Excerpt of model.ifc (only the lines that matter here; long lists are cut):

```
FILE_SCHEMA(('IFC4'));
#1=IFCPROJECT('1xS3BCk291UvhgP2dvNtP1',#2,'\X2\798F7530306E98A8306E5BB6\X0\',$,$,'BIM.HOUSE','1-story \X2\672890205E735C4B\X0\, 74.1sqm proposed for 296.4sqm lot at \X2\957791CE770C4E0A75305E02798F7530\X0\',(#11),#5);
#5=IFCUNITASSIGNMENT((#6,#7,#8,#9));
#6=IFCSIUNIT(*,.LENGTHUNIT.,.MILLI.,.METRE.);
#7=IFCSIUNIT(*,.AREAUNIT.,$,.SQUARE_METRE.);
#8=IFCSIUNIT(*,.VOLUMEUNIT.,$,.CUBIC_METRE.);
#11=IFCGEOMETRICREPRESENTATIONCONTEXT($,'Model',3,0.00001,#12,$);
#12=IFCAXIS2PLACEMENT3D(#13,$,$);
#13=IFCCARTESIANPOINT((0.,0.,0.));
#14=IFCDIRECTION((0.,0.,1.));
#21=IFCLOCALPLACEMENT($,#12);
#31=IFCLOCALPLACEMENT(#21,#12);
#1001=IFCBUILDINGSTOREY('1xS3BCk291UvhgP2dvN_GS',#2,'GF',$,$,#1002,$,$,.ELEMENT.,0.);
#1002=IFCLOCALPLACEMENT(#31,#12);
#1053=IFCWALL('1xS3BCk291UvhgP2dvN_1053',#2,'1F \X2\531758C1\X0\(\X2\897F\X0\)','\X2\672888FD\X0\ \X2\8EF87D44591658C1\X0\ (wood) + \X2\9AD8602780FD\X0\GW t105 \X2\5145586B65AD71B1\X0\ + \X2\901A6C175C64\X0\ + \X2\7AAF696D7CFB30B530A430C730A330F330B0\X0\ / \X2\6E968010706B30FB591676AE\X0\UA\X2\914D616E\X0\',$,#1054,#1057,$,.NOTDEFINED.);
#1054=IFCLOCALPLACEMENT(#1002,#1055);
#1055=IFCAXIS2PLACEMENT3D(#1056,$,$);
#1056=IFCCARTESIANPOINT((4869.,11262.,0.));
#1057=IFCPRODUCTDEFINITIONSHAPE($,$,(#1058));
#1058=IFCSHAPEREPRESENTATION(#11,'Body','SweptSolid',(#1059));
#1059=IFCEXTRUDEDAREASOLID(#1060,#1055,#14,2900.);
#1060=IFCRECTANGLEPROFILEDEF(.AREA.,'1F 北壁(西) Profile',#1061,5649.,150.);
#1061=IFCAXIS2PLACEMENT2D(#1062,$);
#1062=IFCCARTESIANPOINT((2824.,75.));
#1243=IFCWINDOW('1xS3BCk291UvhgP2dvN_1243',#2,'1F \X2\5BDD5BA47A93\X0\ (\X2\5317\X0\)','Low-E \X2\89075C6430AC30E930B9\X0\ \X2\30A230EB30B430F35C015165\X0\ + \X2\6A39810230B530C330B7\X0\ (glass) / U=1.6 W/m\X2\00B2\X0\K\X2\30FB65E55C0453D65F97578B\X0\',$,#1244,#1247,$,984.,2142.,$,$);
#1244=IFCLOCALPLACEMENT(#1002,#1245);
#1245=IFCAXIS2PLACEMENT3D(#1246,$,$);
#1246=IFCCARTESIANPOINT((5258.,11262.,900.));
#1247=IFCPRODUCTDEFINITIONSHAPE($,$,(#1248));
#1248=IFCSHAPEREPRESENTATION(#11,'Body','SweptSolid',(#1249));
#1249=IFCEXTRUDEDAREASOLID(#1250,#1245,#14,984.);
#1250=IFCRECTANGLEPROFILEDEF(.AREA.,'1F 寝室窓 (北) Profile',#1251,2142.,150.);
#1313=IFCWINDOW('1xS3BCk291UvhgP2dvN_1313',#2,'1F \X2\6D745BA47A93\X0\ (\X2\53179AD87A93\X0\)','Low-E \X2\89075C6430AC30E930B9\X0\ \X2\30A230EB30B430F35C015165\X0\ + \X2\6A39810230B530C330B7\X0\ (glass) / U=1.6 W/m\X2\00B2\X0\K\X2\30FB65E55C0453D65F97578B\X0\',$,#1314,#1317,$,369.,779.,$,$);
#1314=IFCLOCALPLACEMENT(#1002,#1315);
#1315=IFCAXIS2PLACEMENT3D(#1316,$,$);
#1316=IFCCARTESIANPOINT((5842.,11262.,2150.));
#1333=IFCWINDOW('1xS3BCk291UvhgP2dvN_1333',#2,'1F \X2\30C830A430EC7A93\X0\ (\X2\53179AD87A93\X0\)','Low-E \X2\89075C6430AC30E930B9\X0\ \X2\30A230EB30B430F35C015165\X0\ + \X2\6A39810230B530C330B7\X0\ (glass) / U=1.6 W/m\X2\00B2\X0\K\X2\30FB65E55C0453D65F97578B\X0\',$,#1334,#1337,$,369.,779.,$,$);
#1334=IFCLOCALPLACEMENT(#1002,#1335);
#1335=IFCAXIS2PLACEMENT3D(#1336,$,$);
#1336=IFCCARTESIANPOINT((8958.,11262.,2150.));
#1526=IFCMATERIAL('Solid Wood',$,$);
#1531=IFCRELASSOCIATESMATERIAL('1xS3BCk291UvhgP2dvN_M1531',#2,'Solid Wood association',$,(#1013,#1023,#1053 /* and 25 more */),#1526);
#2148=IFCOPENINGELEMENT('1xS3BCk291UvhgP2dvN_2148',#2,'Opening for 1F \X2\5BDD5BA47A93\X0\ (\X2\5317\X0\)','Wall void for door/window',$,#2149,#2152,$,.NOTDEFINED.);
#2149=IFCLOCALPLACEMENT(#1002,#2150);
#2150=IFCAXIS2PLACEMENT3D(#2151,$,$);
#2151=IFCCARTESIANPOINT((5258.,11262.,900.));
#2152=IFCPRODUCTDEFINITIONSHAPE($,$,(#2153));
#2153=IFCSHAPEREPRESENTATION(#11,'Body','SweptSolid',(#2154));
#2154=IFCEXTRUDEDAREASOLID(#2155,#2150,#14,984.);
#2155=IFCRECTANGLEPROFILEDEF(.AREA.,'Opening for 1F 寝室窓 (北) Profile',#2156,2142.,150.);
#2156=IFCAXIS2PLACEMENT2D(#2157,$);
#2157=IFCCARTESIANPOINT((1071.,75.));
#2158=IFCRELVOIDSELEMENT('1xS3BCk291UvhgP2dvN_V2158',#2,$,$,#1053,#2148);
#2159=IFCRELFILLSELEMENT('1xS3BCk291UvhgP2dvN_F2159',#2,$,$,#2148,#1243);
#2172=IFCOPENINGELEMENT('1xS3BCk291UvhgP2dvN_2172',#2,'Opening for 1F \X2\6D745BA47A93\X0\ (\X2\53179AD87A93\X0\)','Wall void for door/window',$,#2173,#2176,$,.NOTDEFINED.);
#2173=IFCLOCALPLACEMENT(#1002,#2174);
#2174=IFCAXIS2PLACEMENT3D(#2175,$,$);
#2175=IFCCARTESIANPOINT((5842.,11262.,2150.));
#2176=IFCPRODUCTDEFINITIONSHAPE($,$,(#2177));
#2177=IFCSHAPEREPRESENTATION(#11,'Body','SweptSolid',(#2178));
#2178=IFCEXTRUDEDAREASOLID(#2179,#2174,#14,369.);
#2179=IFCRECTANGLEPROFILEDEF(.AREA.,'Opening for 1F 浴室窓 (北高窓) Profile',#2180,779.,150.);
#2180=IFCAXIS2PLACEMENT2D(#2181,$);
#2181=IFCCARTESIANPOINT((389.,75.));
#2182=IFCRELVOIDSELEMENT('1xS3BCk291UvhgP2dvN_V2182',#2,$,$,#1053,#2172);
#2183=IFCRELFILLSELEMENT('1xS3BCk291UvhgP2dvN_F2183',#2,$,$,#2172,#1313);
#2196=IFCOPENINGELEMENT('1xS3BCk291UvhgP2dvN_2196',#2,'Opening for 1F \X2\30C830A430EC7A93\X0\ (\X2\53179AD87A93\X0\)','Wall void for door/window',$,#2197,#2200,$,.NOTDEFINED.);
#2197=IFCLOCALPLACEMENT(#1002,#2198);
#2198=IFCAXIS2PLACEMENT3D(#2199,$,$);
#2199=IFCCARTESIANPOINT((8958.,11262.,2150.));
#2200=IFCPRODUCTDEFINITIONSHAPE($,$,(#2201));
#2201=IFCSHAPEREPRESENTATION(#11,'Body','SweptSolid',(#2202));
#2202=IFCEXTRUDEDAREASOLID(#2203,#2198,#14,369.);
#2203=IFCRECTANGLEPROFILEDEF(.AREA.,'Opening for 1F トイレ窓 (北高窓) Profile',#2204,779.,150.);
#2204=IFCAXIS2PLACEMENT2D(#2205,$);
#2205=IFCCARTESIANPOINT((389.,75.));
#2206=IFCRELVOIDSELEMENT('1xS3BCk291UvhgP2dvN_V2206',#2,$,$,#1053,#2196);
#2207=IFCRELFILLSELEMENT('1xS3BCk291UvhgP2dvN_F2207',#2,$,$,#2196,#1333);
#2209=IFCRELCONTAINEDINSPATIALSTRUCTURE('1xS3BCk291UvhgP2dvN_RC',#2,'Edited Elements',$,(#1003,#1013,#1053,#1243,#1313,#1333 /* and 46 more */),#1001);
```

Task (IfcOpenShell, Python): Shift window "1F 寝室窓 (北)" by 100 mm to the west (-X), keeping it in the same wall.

```python
import ifcopenshell
import ifcopenshell.api.geometry
import ifcopenshell.util.placement

model = ifcopenshell.open("model.ifc")

window = model.by_guid("1xS3BCk291UvhgP2dvN_1243")
opening = window.FillsVoids[0].RelatingOpeningElement
wall = opening.VoidsElements[0].RelatingBuildingElement

wall_matrix = ifcopenshell.util.placement.get_local_placement(wall.ObjectPlacement)
shift = wall_matrix[:3, 0] * -100.0
before = ifcopenshell.util.placement.get_local_placement(window.ObjectPlacement)[:3, 3].copy()

# The window is not placed relative to its opening, so move both.
for product in (opening, window):
    matrix = ifcopenshell.util.placement.get_local_placement(product.ObjectPlacement)
    matrix[:3, 3] += shift
    ifcopenshell.api.geometry.edit_object_placement(model, product=product, matrix=matrix, is_si=False)

after = ifcopenshell.util.placement.get_local_placement(window.ObjectPlacement)[:3, 3]
print("window moved by", (after - before).round(3) + 0.0)

model.write("model_updated.ifc")
```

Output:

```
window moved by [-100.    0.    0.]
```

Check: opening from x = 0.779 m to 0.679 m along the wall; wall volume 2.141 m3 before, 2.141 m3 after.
